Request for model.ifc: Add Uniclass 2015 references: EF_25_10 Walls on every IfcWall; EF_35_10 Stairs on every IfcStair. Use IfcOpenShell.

First a look at what the model holds.

```python
import ifcopenshell

model = ifcopenshell.open("model.ifc")
print(model.schema)
print("classifications:", [c.Name for c in model.by_type("IfcClassification")])
for ifc_class in ("IfcDoor", "IfcRoof", "IfcStair", "IfcWall", "IfcWindow"):
    print(ifc_class, len(model.by_type(ifc_class)))
```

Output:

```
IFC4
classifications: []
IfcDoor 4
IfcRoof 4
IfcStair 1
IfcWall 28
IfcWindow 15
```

```python
import ifcopenshell
import ifcopenshell.api.classification

model = ifcopenshell.open("model.ifc")

system = ifcopenshell.api.classification.add_classification(model, classification="Uniclass 2015")

codes = {
    "IfcWall": ("EF_25_10", "Walls"),
    "IfcStair": ("EF_35_10", "Stairs"),
}
for ifc_class, (code, name) in codes.items():
    products = model.by_type(ifc_class)
    ifcopenshell.api.classification.add_reference(
        model, products=products, classification=system, identification=code, name=name
    )
    print(code, len(products))

model.write("model_edited.ifc")
```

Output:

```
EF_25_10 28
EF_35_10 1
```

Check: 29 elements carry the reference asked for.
